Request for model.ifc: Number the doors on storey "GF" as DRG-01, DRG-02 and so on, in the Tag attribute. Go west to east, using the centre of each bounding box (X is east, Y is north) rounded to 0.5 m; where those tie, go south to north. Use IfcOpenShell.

First a look at what the model holds.

```python
import ifcopenshell
import ifcopenshell.util.element
import ifcopenshell.util.placement

model = ifcopenshell.open("model.ifc")
print(model.schema)
storey = next(s for s in model.by_type("IfcBuildingStorey") if s.Name == "GF")
doors = [e for e in ifcopenshell.util.element.get_decomposition(storey) if e.is_a("IfcDoor")]
for e in sorted(doors, key=lambda e: e.id()):
    origin = ifcopenshell.util.placement.get_local_placement(e.ObjectPlacement)[:3, 3]
    print(e.id(), e.Tag, e.Name, origin.round(2) + 0.0, sep=" | ")
```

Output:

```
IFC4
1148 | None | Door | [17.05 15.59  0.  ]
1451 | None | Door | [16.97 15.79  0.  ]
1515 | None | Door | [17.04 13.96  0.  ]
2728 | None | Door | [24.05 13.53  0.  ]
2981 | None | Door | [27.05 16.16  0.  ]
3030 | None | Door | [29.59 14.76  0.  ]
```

```python
import ifcopenshell
import ifcopenshell.geom
import ifcopenshell.util.element
import ifcopenshell.util.shape

model = ifcopenshell.open("model.ifc")
settings = ifcopenshell.geom.settings()
settings.set("use-world-coords", True)


def centre(element):
    shape = ifcopenshell.geom.create_shape(settings, element)
    return ifcopenshell.util.shape.get_bbox_centroid(shape.geometry)


storey = next(s for s in model.by_type("IfcBuildingStorey") if s.Name == "GF")
doors = [e for e in ifcopenshell.util.element.get_decomposition(storey) if e.is_a("IfcDoor")]

# Insertion points can sit at a corner or the storey origin, so sort by the geometry (in metres).
centres = {e: centre(e) for e in doors}
doors.sort(key=lambda e: (round(centres[e][0] / 0.5), centres[e][1]))

for i, e in enumerate(doors, start=1):
    number = f"DRG-{i:02d}"
    e.Tag = number
    print(e.id(), number)

model.write("model_updated.ifc")
```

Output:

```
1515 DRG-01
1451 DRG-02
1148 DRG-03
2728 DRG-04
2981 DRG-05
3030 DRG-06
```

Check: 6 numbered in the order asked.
